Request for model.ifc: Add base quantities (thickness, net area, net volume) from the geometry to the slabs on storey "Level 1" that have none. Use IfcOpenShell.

First a look at what the model holds.

```python
import ifcopenshell
import ifcopenshell.util.element
import ifcopenshell.util.unit

model = ifcopenshell.open("model.ifc")
print(model.schema)
for unit_type in ("LENGTHUNIT", "AREAUNIT", "VOLUMEUNIT"):
    print(unit_type, ifcopenshell.util.unit.calculate_unit_scale(model, unit_type))
storey = next(s for s in model.by_type("IfcBuildingStorey") if s.Name == "Level 1")
slabs = [e for e in ifcopenshell.util.element.get_decomposition(storey) if e.is_a("IfcSlab")]
for e in sorted(slabs, key=lambda e: e.id()):
    print(e.id(), e.is_a(), e.Name, list(ifcopenshell.util.element.get_psets(e, qtos_only=True)), sep=" | ")
```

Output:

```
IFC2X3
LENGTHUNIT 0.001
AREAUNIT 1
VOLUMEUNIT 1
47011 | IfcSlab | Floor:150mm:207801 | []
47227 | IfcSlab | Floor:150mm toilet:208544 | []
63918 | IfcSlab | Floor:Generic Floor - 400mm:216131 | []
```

```python
import ifcopenshell
import ifcopenshell.api.pset
import ifcopenshell.geom
import ifcopenshell.util.element
import ifcopenshell.util.shape
import ifcopenshell.util.unit

model = ifcopenshell.open("model.ifc")
unit_scale = ifcopenshell.util.unit.calculate_unit_scale(model)
area_scale = ifcopenshell.util.unit.calculate_unit_scale(model, "AREAUNIT")
volume_scale = ifcopenshell.util.unit.calculate_unit_scale(model, "VOLUMEUNIT")
settings = ifcopenshell.geom.settings()

storey = next(s for s in model.by_type("IfcBuildingStorey") if s.Name == "Level 1")
slabs = [e for e in ifcopenshell.util.element.get_decomposition(storey) if e.is_a("IfcSlab")]

for e in sorted(slabs, key=lambda e: e.id()):
    if ifcopenshell.util.element.get_psets(e, qtos_only=True, should_inherit=False):
        continue
    # Geometry comes back in metres, in the element's own axes.
    shape = ifcopenshell.geom.create_shape(settings, e)
    values = {
        "Width": ifcopenshell.util.shape.get_z(shape.geometry) / unit_scale,
        "NetArea": ifcopenshell.util.shape.get_footprint_area(shape.geometry) / area_scale,
        "NetVolume": ifcopenshell.util.shape.get_volume(shape.geometry) / volume_scale,
    }
    qto = ifcopenshell.api.pset.add_qto(model, product=e, name="BaseQuantities")
    ifcopenshell.api.pset.edit_qto(model, qto=qto, properties=values)
    print(e.id(), {k: round(v, 3) for k, v in values.items()})

model.write("model_rev.ifc")
```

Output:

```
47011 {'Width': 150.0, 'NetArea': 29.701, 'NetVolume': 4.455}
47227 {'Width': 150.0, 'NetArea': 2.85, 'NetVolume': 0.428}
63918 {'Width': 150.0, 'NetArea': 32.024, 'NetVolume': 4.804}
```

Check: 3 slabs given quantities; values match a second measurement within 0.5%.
